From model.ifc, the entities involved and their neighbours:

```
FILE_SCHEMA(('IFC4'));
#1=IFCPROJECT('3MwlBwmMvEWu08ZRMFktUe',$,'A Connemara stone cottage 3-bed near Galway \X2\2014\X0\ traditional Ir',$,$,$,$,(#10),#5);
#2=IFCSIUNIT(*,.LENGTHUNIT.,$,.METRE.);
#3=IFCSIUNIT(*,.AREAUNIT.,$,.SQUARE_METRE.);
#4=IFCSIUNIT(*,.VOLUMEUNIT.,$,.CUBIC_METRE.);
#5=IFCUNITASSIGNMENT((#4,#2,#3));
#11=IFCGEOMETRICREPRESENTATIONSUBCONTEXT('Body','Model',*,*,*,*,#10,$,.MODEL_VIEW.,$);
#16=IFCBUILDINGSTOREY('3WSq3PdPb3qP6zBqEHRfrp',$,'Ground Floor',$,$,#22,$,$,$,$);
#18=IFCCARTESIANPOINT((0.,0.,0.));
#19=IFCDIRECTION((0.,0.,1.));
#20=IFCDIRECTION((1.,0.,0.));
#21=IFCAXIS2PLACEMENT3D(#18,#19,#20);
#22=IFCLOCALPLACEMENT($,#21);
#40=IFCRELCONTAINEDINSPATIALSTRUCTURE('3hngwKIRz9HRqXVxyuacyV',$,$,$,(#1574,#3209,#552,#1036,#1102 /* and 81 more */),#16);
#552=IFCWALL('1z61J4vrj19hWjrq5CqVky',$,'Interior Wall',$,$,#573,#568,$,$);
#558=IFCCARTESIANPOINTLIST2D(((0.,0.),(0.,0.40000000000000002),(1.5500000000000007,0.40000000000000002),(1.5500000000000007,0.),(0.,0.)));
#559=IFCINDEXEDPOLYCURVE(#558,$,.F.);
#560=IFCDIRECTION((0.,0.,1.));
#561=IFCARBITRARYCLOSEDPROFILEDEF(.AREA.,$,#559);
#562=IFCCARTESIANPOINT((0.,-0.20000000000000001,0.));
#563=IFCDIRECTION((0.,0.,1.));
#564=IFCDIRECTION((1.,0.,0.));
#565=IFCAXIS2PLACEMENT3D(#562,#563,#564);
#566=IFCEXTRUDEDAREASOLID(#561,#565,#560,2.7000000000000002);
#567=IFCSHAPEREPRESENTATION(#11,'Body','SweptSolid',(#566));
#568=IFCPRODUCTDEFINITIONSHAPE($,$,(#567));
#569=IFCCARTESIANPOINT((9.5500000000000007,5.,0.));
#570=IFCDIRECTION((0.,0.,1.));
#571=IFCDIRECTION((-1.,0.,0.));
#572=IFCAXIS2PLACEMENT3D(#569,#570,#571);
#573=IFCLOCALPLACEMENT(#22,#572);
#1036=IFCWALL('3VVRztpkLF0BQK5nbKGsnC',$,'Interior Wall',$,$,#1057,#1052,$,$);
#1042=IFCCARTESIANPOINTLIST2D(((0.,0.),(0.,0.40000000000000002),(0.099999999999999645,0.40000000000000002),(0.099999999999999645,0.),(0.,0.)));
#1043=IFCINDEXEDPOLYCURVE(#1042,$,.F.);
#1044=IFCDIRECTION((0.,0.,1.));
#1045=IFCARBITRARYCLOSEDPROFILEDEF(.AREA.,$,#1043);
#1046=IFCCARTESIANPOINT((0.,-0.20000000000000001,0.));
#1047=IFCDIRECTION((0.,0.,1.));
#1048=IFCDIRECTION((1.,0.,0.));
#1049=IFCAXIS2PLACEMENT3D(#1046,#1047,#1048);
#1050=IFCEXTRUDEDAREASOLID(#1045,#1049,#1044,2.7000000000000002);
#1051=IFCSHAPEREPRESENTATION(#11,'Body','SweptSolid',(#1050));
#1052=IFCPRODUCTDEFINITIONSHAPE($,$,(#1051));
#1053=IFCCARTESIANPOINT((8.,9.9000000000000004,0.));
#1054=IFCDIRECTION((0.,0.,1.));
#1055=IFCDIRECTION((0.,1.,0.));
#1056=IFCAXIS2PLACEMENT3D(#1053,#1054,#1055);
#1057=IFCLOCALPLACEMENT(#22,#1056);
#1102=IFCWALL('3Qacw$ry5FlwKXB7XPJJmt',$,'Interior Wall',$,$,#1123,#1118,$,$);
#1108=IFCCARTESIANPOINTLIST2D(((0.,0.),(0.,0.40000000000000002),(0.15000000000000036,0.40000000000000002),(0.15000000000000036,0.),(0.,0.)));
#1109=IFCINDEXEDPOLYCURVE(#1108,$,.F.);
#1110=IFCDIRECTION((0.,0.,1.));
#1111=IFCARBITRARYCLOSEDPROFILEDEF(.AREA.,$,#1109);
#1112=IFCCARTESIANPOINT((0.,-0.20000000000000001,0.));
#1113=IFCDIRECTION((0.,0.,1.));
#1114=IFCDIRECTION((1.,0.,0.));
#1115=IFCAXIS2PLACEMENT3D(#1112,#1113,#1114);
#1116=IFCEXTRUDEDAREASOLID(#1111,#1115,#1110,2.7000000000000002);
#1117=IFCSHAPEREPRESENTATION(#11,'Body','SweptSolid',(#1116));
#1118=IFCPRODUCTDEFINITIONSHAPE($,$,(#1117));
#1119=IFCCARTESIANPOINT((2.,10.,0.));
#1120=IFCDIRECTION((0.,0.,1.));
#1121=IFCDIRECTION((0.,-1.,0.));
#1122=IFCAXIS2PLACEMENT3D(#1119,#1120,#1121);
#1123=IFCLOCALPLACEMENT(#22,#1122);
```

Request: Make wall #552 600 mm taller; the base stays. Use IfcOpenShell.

```python
import ifcopenshell
import ifcopenshell.geom
import ifcopenshell.util.representation
import ifcopenshell.util.shape
import ifcopenshell.util.unit

model = ifcopenshell.open("model.ifc")
unit_scale = ifcopenshell.util.unit.calculate_unit_scale(model)
settings = ifcopenshell.geom.settings()


def volume(element):
    """Net volume in cubic metres, openings subtracted."""
    shape = ifcopenshell.geom.create_shape(settings, element)
    return ifcopenshell.util.shape.get_volume(shape.geometry)


wall = model.by_guid("1z61J4vrj19hWjrq5CqVky")
before = volume(wall)

body = ifcopenshell.util.representation.get_representation(wall, "Model", "Body")
solid = body.Items[0]
old_height = solid.Depth
solid.Depth += 0.6 / unit_scale
after = volume(wall)

print(f"height {old_height:g} -> {solid.Depth:g}, volume {before:.3f} -> {after:.3f} m3")

model.write("model_updated.ifc")
```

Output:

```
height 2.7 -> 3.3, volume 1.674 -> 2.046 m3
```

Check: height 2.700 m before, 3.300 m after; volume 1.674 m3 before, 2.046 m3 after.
